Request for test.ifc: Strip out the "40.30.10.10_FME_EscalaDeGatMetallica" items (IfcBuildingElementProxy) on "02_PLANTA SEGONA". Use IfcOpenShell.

First a look at what the model holds.

```python
import ifcopenshell
import ifcopenshell.util.element

model = ifcopenshell.open("test.ifc")
print(model.schema)
storey = next(s for s in model.by_type("IfcBuildingStorey") if s.Name == "02_PLANTA SEGONA")
proxies = [e for e in ifcopenshell.util.element.get_decomposition(storey) if e.is_a("IfcBuildingElementProxy")]
seen = {}
for e in proxies:
    element_type = ifcopenshell.util.element.get_type(e)
    name = element_type.Name if element_type not in (None, e) else None
    seen[name] = seen.get(name, 0) + 1
for name, count in sorted(seen.items(), key=str):
    print(count, "x", name)
```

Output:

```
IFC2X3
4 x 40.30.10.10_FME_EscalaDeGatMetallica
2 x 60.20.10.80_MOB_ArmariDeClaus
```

```python
import ifcopenshell
import ifcopenshell.api.root
import ifcopenshell.util.element

model = ifcopenshell.open("test.ifc")

storey = next(s for s in model.by_type("IfcBuildingStorey") if s.Name == "02_PLANTA SEGONA")
proxies = [e for e in ifcopenshell.util.element.get_decomposition(storey) if e.is_a("IfcBuildingElementProxy")]
targets = [e for e in proxies if (t := ifcopenshell.util.element.get_type(e)) not in (None, e) and t.Name == "40.30.10.10_FME_EscalaDeGatMetallica"]

for e in targets:
    ifcopenshell.api.root.remove_product(model, product=e)
print(len(targets), "removed")

model.write("test_v2.ifc")
```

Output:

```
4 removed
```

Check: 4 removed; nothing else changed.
